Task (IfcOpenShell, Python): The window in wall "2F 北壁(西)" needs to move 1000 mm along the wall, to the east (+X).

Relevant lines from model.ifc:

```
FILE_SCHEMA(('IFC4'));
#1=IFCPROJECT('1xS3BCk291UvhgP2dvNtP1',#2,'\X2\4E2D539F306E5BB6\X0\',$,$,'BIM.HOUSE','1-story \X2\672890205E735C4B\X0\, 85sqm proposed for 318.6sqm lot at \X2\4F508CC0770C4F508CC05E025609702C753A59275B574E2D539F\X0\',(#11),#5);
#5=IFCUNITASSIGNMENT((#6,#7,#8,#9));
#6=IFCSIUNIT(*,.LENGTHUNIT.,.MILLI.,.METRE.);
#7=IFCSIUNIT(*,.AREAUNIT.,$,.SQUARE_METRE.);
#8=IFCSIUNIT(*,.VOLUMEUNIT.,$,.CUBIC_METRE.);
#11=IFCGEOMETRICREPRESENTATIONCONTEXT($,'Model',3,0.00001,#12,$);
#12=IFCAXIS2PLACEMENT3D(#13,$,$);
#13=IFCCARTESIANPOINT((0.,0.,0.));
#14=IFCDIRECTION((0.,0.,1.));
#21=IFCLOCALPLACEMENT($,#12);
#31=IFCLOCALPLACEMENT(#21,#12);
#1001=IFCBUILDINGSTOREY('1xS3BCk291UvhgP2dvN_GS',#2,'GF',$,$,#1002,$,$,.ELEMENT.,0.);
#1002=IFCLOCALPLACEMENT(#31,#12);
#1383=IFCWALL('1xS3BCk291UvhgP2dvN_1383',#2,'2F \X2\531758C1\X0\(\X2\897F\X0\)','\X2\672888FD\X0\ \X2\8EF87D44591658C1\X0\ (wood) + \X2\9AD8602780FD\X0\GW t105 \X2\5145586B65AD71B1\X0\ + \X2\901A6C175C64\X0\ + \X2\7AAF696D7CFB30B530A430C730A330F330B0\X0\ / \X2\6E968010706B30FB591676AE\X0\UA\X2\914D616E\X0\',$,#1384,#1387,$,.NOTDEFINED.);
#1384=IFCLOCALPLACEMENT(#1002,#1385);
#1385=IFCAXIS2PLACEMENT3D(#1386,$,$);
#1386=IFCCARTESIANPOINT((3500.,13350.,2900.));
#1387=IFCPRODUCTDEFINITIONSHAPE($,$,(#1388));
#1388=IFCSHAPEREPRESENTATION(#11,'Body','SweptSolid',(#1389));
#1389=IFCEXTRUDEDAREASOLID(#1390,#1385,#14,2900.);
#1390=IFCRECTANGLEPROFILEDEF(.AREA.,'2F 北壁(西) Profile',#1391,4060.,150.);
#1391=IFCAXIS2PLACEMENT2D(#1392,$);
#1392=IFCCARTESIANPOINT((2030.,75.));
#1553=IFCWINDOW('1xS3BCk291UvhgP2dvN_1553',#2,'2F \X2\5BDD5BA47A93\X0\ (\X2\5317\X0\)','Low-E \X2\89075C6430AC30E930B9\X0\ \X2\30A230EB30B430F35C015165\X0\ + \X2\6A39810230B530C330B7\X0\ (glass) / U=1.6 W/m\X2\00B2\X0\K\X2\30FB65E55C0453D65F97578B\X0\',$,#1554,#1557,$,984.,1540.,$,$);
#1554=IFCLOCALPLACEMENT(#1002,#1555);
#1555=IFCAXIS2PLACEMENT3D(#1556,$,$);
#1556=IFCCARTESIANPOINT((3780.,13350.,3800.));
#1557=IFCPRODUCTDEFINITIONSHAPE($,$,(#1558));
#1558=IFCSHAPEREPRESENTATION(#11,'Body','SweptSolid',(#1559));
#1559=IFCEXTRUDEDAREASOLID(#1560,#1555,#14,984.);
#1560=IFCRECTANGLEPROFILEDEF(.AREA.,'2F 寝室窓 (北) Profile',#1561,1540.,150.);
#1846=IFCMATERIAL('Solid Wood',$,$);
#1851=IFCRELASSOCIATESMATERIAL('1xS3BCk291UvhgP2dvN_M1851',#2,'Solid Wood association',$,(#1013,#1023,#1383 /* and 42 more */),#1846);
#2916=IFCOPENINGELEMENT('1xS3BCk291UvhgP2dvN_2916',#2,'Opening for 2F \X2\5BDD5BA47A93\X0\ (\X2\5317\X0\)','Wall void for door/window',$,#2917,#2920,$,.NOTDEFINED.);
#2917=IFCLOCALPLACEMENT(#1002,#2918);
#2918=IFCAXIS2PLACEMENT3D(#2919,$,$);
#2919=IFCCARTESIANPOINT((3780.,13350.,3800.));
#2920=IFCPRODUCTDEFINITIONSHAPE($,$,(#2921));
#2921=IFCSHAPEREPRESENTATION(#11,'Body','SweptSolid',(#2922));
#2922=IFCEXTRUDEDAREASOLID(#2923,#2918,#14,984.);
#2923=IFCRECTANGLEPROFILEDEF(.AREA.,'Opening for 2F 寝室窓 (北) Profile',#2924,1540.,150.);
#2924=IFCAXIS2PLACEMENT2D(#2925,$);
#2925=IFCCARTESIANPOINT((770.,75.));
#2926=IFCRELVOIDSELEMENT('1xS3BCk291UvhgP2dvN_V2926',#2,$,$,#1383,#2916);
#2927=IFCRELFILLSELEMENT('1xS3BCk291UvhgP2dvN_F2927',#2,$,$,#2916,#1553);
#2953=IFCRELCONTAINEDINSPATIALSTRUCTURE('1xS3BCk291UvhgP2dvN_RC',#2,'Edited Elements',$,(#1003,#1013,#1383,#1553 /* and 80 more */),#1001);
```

```python
import ifcopenshell
import ifcopenshell.api.geometry
import ifcopenshell.util.placement

model = ifcopenshell.open("model.ifc")

window = model.by_guid("1xS3BCk291UvhgP2dvN_1553")
opening = window.FillsVoids[0].RelatingOpeningElement
wall = opening.VoidsElements[0].RelatingBuildingElement

wall_matrix = ifcopenshell.util.placement.get_local_placement(wall.ObjectPlacement)
shift = wall_matrix[:3, 0] * 1000.0
before = ifcopenshell.util.placement.get_local_placement(window.ObjectPlacement)[:3, 3].copy()

# The window is not placed relative to its opening, so move both.
for product in (opening, window):
    matrix = ifcopenshell.util.placement.get_local_placement(product.ObjectPlacement)
    matrix[:3, 3] += shift
    ifcopenshell.api.geometry.edit_object_placement(model, product=product, matrix=matrix, is_si=False)

after = ifcopenshell.util.placement.get_local_placement(window.ObjectPlacement)[:3, 3]
print("window moved by", (after - before).round(3) + 0.0)

model.write("model_updated.ifc")
```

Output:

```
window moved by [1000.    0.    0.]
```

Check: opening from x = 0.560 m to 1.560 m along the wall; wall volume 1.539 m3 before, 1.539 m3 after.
